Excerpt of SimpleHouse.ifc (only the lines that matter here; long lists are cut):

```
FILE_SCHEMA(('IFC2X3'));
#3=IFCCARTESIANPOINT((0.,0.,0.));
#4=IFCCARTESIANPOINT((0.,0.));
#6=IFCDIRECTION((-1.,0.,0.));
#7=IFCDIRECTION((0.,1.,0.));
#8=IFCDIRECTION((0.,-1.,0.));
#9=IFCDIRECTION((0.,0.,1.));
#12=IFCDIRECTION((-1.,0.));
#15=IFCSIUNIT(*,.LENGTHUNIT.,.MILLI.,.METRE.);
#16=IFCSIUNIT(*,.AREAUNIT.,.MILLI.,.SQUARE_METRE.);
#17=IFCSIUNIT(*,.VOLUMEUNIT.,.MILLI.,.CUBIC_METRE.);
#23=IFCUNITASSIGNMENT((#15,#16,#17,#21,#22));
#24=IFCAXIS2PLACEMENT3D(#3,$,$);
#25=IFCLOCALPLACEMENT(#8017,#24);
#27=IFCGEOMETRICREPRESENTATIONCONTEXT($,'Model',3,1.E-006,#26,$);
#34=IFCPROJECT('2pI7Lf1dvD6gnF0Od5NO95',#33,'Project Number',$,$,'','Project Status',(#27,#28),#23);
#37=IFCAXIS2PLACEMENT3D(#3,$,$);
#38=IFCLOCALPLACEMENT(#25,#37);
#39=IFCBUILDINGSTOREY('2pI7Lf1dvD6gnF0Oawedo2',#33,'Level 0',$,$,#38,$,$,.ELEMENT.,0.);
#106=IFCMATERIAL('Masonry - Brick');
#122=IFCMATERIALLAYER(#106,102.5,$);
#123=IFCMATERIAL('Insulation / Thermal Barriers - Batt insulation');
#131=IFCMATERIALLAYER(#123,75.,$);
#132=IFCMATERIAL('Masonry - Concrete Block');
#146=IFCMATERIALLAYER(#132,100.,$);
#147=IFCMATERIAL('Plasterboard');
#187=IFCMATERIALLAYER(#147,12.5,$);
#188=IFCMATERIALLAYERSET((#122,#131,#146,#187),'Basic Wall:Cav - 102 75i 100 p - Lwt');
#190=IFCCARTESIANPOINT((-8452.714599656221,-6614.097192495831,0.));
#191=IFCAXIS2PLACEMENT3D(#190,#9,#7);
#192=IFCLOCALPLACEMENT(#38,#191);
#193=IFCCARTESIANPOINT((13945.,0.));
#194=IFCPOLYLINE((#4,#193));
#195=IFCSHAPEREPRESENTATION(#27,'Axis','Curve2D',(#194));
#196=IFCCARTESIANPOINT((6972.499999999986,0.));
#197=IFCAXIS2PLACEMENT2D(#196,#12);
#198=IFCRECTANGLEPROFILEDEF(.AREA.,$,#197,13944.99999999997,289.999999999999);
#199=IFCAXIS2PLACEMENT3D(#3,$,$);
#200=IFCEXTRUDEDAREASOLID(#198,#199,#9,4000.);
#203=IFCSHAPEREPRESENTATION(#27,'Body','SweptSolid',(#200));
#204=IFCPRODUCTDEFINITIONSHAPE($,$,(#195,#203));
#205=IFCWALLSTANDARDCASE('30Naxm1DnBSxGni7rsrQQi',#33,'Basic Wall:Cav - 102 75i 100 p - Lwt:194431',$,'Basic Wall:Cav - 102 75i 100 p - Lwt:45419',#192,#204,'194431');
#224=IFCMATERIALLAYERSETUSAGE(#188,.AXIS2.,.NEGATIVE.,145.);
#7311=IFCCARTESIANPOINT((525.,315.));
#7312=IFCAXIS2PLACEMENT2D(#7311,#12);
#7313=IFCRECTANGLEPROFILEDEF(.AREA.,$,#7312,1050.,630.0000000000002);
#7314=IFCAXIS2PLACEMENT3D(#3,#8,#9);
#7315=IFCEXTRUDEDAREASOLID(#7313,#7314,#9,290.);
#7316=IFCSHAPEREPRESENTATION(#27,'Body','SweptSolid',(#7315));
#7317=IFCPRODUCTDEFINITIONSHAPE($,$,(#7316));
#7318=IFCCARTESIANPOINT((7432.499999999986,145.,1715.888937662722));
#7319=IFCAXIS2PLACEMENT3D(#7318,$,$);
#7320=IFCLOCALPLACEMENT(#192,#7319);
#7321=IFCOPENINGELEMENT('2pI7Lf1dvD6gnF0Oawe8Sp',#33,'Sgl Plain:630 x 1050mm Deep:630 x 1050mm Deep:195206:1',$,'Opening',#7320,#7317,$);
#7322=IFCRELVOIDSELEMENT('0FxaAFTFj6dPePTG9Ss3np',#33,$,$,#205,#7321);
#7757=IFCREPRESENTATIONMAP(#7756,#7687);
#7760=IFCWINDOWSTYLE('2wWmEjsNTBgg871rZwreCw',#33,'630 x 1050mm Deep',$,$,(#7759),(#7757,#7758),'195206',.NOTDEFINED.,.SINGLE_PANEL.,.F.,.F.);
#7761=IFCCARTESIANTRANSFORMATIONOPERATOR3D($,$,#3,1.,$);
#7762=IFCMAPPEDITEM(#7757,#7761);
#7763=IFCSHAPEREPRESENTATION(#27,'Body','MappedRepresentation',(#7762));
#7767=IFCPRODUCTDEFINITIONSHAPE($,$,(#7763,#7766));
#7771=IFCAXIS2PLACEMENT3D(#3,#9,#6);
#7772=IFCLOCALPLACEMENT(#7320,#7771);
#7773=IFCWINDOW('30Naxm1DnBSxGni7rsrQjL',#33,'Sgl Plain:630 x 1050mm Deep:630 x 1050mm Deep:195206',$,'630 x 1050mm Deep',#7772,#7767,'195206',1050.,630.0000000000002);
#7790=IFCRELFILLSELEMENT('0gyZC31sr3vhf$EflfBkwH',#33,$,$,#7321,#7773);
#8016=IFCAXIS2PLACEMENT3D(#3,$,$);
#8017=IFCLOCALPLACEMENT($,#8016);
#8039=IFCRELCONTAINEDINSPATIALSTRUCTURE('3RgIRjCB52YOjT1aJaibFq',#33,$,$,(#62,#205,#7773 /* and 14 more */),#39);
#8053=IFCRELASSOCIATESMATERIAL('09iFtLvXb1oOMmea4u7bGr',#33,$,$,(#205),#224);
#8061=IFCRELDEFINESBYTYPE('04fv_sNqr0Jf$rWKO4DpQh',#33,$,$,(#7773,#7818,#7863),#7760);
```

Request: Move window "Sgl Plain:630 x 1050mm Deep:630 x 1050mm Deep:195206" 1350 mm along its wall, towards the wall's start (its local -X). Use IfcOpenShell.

```python
import ifcopenshell
import ifcopenshell.api.geometry
import ifcopenshell.util.placement
import ifcopenshell.util.unit

model = ifcopenshell.open("SimpleHouse.ifc")
unit_scale = ifcopenshell.util.unit.calculate_unit_scale(model)

window = model.by_id(7773)
opening = window.FillsVoids[0].RelatingOpeningElement
wall = opening.VoidsElements[0].RelatingBuildingElement

wall_matrix = ifcopenshell.util.placement.get_local_placement(wall.ObjectPlacement)
shift = wall_matrix[:3, 0] * -1.35 / unit_scale
before = ifcopenshell.util.placement.get_local_placement(window.ObjectPlacement)[:3, 3].copy()

# The window is placed relative to its opening, so it follows when the opening moves.
matrix = ifcopenshell.util.placement.get_local_placement(opening.ObjectPlacement)
matrix[:3, 3] += shift
ifcopenshell.api.geometry.edit_object_placement(
    model, product=opening, matrix=matrix, is_si=False, should_transform_children=True
)

after = ifcopenshell.util.placement.get_local_placement(window.ObjectPlacement)[:3, 3]
print("window moved by", (after - before).round(3) + 0.0)

model.write("SimpleHouse_updated.ifc")
```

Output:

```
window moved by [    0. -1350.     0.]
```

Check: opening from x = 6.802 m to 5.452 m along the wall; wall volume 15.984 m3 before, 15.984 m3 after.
